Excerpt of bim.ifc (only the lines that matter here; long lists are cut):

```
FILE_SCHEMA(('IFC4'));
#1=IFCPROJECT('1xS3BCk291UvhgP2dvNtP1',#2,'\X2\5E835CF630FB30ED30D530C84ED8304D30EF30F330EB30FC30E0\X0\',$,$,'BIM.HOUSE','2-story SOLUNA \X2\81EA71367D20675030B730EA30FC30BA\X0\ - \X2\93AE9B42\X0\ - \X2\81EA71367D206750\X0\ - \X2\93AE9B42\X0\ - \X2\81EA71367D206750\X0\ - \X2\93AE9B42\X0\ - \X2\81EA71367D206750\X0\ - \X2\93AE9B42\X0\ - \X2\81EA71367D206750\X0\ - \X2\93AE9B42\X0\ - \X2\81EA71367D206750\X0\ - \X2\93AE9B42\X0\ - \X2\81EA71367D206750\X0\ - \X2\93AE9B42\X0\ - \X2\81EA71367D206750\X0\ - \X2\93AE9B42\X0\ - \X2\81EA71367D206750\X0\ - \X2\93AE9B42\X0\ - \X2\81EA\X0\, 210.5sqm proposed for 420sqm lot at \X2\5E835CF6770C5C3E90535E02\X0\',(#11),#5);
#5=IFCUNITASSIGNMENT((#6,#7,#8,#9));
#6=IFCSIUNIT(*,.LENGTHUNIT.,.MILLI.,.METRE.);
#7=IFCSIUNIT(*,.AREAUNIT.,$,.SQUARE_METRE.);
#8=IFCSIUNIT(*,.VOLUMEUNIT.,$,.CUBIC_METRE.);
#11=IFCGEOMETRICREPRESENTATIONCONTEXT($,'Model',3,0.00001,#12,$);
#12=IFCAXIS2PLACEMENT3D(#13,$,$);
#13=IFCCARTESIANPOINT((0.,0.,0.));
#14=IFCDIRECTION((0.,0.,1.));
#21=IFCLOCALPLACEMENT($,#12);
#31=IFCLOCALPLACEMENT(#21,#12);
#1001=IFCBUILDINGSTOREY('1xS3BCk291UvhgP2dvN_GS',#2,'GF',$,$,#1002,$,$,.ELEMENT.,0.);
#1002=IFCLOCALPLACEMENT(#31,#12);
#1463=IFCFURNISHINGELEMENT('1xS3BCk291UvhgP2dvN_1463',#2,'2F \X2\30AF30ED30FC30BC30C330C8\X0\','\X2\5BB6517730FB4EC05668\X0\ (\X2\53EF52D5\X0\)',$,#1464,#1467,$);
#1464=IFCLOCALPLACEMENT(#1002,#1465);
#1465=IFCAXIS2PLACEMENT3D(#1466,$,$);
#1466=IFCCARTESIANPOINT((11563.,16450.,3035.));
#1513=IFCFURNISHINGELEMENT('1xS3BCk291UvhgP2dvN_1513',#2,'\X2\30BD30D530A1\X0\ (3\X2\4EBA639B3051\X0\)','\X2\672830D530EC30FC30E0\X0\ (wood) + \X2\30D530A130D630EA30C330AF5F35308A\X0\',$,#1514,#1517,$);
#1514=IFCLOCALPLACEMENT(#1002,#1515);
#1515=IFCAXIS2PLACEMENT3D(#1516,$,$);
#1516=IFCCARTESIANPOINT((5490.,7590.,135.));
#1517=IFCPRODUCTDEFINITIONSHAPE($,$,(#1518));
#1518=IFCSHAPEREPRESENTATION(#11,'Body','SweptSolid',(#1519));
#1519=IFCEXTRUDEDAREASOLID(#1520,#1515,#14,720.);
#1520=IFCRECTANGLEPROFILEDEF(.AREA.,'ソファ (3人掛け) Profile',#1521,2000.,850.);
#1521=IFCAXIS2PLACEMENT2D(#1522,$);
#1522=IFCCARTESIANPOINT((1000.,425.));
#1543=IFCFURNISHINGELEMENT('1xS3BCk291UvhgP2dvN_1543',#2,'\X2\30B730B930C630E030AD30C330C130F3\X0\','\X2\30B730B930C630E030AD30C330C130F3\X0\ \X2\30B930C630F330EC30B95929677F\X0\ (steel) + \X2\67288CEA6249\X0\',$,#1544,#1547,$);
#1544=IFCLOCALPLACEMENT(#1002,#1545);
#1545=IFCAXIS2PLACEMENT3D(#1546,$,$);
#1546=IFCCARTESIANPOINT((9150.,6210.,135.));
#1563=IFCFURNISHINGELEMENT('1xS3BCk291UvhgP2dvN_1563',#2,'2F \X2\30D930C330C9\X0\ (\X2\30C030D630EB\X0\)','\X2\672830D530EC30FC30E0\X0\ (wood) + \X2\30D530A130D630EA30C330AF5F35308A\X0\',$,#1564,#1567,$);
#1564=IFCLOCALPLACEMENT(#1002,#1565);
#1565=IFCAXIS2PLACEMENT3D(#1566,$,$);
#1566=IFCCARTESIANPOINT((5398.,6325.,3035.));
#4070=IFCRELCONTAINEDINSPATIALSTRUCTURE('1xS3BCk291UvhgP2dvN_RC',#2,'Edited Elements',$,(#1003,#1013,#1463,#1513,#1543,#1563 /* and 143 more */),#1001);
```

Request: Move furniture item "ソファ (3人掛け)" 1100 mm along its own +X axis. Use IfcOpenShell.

```python
import ifcopenshell
import ifcopenshell.api.geometry
import ifcopenshell.util.placement
import ifcopenshell.util.unit

model = ifcopenshell.open("bim.ifc")
unit_scale = ifcopenshell.util.unit.calculate_unit_scale(model)

item = model.by_guid("1xS3BCk291UvhgP2dvN_1513")
matrix = ifcopenshell.util.placement.get_local_placement(item.ObjectPlacement)
matrix[:3, 3] += matrix[:3, 0] * 1.1 / unit_scale
ifcopenshell.api.geometry.edit_object_placement(model, product=item, matrix=matrix, is_si=False)

print(ifcopenshell.util.placement.get_local_placement(item.ObjectPlacement).round(3) + 0.0)

model.write("bim_rev.ifc")
```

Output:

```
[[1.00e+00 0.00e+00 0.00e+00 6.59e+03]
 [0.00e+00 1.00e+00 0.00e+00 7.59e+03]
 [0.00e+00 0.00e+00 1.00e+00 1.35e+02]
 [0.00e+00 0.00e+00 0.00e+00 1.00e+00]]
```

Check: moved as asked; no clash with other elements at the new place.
